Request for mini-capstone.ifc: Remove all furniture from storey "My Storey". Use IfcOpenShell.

First a look at what the model holds.

```python
import ifcopenshell
import ifcopenshell.util.element

model = ifcopenshell.open("mini-capstone.ifc")
print(model.schema)
storey = next(s for s in model.by_type("IfcBuildingStorey") if s.Name == "My Storey")
furniture = [e for e in ifcopenshell.util.element.get_decomposition(storey) if e.is_a("IfcFurnishingElement")]
seen = {}
for e in furniture:
    element_type = ifcopenshell.util.element.get_type(e)
    name = element_type.Name if element_type not in (None, e) else None
    seen[name] = seen.get(name, 0) + 1
for name, count in sorted(seen.items(), key=str):
    print(count, "x", name)
```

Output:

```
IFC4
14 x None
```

```python
import ifcopenshell
import ifcopenshell.api.root
import ifcopenshell.util.element

model = ifcopenshell.open("mini-capstone.ifc")

storey = next(s for s in model.by_type("IfcBuildingStorey") if s.Name == "My Storey")
furniture = [e for e in ifcopenshell.util.element.get_decomposition(storey) if e.is_a("IfcFurnishingElement")]

for e in furniture:
    ifcopenshell.api.root.remove_product(model, product=e)
print(len(furniture), "removed")

model.write("mini-capstone-out.ifc")
```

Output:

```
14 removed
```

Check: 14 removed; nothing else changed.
